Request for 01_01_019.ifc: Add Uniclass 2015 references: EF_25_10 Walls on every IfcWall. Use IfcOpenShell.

First a look at what the model holds.

```python
import ifcopenshell

model = ifcopenshell.open("01_01_019.ifc")
print(model.schema)
print("classifications:", [c.Name for c in model.by_type("IfcClassification")])
for ifc_class in ("IfcDoor", "IfcRoof", "IfcStair", "IfcWall", "IfcWindow"):
    print(ifc_class, len(model.by_type(ifc_class)))
```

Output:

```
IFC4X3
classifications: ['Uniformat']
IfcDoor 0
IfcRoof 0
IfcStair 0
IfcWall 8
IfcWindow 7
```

```python
import ifcopenshell
import ifcopenshell.api.classification

model = ifcopenshell.open("01_01_019.ifc")

system = ifcopenshell.api.classification.add_classification(model, classification="Uniclass 2015")

codes = {
    "IfcWall": ("EF_25_10", "Walls"),
}
for ifc_class, (code, name) in codes.items():
    products = model.by_type(ifc_class)
    ifcopenshell.api.classification.add_reference(
        model, products=products, classification=system, identification=code, name=name
    )
    print(code, len(products))

model.write("01_01_019_edited.ifc")
```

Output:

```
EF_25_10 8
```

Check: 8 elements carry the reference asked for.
